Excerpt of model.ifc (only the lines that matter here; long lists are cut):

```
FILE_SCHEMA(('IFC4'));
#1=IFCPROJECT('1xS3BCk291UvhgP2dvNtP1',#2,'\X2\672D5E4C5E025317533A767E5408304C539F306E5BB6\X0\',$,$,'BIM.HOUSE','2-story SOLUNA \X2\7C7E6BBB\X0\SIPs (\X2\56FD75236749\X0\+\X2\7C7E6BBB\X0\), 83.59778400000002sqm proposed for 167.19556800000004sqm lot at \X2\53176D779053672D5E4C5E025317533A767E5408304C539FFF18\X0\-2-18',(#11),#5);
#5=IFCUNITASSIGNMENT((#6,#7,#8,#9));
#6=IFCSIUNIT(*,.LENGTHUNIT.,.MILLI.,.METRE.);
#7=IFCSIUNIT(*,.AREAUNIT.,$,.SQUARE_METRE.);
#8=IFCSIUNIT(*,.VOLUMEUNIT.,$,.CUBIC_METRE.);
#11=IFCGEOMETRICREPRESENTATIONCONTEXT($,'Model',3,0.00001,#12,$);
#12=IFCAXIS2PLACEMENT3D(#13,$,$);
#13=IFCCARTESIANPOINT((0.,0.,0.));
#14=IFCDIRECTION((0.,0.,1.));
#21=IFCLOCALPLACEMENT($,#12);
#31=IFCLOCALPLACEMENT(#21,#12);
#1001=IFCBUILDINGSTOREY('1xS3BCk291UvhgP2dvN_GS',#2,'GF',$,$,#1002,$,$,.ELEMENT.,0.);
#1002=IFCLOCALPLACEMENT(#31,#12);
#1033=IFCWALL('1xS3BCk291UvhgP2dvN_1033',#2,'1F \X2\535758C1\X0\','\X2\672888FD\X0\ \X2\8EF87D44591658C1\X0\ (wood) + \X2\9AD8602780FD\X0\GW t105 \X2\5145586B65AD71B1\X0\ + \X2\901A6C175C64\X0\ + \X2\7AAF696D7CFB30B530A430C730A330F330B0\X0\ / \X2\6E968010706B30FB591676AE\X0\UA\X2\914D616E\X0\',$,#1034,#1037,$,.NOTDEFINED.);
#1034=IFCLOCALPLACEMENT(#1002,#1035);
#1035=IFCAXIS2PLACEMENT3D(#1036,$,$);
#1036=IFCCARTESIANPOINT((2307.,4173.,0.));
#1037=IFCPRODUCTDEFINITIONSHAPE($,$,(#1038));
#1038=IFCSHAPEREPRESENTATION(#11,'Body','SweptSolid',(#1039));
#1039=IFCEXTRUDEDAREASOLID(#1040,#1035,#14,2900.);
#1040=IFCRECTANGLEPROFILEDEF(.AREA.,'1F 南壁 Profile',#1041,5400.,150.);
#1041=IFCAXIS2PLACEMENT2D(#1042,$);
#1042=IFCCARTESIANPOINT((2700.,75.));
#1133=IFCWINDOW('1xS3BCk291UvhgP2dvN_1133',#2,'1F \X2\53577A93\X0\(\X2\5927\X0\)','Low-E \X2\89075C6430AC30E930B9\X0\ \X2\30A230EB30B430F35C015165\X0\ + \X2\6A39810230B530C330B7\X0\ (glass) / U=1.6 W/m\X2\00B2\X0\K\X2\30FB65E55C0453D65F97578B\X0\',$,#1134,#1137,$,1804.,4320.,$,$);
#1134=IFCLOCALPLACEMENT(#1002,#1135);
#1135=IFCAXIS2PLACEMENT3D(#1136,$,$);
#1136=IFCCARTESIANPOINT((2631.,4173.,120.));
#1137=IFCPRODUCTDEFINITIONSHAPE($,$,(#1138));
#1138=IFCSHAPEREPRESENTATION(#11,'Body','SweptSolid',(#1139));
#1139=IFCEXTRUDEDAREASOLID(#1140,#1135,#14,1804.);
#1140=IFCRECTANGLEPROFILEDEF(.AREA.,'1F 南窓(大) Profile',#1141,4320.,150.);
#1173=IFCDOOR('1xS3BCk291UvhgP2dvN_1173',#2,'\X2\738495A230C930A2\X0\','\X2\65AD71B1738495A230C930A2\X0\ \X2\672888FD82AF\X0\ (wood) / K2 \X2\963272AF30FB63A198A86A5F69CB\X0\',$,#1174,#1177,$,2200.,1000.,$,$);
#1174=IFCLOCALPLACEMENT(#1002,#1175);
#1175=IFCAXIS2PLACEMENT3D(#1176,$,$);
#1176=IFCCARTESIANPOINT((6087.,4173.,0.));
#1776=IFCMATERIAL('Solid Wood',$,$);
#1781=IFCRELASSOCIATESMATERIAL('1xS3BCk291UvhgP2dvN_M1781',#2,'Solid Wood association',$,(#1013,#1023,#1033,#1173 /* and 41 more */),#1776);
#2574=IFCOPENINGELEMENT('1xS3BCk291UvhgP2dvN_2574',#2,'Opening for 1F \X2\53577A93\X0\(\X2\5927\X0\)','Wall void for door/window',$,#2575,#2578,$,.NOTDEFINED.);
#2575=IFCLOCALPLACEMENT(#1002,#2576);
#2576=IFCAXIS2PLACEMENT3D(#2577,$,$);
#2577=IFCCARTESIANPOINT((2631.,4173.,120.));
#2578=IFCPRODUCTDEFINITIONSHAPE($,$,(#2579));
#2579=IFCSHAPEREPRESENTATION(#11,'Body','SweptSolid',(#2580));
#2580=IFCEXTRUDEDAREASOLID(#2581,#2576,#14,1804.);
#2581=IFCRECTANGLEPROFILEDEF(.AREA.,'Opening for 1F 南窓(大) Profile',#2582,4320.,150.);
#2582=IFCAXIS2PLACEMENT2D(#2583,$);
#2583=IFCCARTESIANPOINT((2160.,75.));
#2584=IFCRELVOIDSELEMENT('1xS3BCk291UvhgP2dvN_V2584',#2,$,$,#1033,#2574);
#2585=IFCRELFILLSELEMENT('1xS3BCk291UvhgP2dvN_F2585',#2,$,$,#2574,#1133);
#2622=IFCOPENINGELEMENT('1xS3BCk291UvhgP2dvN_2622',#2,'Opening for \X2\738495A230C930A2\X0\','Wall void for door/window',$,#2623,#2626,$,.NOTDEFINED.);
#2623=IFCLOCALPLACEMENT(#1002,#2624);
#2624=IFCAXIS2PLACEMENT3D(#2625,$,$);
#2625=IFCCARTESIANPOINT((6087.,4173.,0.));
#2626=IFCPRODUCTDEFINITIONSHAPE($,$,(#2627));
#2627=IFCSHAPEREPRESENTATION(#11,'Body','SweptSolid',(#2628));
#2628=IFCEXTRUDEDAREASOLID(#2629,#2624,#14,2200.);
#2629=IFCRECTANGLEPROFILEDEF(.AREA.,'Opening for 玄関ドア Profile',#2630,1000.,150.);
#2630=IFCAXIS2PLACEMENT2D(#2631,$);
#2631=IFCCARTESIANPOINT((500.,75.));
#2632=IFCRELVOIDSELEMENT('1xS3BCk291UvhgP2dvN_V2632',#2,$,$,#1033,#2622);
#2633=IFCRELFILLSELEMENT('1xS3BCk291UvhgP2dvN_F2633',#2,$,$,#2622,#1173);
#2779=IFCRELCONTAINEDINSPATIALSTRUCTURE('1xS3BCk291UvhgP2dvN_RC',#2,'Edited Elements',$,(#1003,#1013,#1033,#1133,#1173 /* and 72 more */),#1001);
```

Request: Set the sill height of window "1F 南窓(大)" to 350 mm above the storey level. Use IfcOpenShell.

```python
import numpy as np
import ifcopenshell
import ifcopenshell.api.geometry
import ifcopenshell.geom
import ifcopenshell.util.element
import ifcopenshell.util.placement
import ifcopenshell.util.shape
import ifcopenshell.util.unit

model = ifcopenshell.open("model.ifc")
unit_scale = ifcopenshell.util.unit.calculate_unit_scale(model)

window = model.by_guid("1xS3BCk291UvhgP2dvN_1133")
opening = window.FillsVoids[0].RelatingOpeningElement
storey = ifcopenshell.util.element.get_container(window, ifc_class="IfcBuildingStorey")
level = ifcopenshell.util.placement.get_local_placement(storey.ObjectPlacement)[2, 3]

# The opening's origin need not be at the sill, so measure its lowest point.
shape = ifcopenshell.geom.create_shape(ifcopenshell.geom.settings(), opening)
bottom = ifcopenshell.util.shape.get_shape_bottom_elevation(shape, shape.geometry) / unit_scale
dz = level + 0.35 / unit_scale - bottom

shift = np.array([0.0, 0.0, dz])
# The window is not placed relative to its opening, so move both.
for product in (opening, window):
    matrix = ifcopenshell.util.placement.get_local_placement(product.ObjectPlacement)
    matrix[:3, 3] += shift
    ifcopenshell.api.geometry.edit_object_placement(model, product=product, matrix=matrix, is_si=False)

print(f"moved by {dz * unit_scale:+.3f} m")

model.write("model_edited.ifc")
```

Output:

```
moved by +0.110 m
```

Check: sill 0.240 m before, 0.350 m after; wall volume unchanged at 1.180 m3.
